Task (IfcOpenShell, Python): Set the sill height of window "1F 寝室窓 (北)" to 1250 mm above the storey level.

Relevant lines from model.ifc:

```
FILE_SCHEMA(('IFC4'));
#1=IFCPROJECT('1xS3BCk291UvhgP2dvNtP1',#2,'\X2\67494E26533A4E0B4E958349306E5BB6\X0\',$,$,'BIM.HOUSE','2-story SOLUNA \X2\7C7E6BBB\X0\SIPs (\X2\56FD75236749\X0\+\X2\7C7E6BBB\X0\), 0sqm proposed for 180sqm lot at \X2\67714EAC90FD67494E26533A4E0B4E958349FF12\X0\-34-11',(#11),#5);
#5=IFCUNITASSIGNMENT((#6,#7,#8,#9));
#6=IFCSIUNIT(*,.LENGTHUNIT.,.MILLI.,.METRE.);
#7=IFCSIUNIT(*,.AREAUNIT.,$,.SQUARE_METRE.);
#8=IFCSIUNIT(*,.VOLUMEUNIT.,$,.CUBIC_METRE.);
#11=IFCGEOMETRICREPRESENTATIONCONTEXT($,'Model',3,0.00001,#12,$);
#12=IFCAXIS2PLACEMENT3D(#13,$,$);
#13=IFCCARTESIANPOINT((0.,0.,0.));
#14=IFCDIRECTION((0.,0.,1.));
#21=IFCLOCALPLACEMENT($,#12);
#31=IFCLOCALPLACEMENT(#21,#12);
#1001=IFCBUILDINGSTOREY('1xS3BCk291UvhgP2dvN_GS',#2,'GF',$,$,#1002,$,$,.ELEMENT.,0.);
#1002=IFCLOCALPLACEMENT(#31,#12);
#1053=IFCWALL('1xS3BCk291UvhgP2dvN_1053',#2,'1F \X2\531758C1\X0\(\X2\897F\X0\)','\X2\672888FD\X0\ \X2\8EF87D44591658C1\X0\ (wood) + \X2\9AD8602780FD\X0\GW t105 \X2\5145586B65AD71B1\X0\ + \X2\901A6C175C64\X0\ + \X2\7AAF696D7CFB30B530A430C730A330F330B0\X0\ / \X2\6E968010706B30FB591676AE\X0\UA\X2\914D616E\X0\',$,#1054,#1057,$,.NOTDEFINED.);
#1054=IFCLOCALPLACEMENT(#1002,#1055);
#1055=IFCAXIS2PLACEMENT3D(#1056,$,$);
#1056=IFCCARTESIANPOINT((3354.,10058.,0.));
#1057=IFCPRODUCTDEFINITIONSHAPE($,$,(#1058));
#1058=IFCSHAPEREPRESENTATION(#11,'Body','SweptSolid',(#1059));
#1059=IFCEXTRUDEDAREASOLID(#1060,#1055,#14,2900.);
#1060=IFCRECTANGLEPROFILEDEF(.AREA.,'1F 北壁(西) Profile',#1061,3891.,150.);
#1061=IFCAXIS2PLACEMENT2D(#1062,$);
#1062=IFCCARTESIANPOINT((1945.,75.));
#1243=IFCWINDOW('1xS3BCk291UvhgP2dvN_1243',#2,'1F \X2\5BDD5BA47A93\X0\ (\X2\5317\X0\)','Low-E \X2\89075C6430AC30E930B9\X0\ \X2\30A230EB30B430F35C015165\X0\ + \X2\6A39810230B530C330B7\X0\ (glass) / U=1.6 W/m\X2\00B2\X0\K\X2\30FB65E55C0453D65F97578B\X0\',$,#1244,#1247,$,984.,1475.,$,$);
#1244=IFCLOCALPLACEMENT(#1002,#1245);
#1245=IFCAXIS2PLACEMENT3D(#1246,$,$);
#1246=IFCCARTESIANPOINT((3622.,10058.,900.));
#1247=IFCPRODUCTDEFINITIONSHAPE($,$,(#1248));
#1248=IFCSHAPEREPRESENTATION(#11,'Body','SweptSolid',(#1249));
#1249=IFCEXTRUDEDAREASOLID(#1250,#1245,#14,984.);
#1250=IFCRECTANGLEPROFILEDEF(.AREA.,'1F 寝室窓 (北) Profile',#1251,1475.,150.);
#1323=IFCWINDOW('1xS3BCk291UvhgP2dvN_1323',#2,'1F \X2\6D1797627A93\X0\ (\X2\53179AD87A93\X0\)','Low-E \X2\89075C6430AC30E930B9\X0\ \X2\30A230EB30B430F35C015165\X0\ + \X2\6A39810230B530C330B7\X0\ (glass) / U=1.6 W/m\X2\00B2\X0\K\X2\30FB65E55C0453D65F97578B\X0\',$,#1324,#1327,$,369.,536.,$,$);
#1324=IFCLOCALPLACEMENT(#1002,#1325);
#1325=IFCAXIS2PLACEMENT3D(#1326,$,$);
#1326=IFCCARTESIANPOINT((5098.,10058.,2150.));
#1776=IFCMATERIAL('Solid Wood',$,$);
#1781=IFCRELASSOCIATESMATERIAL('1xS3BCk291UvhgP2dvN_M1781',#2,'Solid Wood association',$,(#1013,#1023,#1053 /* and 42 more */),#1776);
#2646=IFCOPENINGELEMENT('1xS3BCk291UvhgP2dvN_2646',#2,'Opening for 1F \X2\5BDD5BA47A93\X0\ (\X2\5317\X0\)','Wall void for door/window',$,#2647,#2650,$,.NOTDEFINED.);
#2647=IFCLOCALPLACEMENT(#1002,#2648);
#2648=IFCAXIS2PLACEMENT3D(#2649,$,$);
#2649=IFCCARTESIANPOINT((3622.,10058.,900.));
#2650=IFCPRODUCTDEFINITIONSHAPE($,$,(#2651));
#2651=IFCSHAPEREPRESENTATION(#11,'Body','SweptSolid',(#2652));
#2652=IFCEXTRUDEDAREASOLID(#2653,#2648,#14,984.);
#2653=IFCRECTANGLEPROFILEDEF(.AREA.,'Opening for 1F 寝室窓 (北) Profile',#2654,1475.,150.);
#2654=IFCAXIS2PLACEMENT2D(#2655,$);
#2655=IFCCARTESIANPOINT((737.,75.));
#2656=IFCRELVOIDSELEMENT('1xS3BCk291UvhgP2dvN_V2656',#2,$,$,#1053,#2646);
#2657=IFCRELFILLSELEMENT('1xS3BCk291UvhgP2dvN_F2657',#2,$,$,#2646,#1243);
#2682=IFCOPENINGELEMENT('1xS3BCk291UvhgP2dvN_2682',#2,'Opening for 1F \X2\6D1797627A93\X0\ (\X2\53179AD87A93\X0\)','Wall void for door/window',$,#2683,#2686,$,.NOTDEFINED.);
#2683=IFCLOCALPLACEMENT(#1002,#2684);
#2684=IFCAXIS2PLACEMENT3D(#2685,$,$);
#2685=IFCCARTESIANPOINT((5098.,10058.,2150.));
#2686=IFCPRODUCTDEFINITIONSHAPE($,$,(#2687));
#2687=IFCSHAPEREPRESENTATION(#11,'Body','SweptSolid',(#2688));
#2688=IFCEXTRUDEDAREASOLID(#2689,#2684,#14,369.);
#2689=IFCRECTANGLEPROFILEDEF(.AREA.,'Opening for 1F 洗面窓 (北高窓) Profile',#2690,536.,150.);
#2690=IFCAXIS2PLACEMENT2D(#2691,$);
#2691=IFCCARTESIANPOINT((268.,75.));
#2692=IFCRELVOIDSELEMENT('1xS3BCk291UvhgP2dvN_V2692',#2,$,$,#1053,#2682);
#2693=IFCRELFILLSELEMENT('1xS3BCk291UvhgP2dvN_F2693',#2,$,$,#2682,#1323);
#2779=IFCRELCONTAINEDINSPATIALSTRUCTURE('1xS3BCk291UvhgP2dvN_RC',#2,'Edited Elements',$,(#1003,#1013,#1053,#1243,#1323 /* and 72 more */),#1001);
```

```python
import numpy as np
import ifcopenshell
import ifcopenshell.api.geometry
import ifcopenshell.geom
import ifcopenshell.util.element
import ifcopenshell.util.placement
import ifcopenshell.util.shape
import ifcopenshell.util.unit

model = ifcopenshell.open("model.ifc")
unit_scale = ifcopenshell.util.unit.calculate_unit_scale(model)

window = model.by_guid("1xS3BCk291UvhgP2dvN_1243")
opening = window.FillsVoids[0].RelatingOpeningElement
storey = ifcopenshell.util.element.get_container(window, ifc_class="IfcBuildingStorey")
level = ifcopenshell.util.placement.get_local_placement(storey.ObjectPlacement)[2, 3]

# The opening's origin need not be at the sill, so measure its lowest point.
shape = ifcopenshell.geom.create_shape(ifcopenshell.geom.settings(), opening)
bottom = ifcopenshell.util.shape.get_shape_bottom_elevation(shape, shape.geometry) / unit_scale
dz = level + 1250.0 - bottom

shift = np.array([0.0, 0.0, dz])
# The window is not placed relative to its opening, so move both.
for product in (opening, window):
    matrix = ifcopenshell.util.placement.get_local_placement(product.ObjectPlacement)
    matrix[:3, 3] += shift
    ifcopenshell.api.geometry.edit_object_placement(model, product=product, matrix=matrix, is_si=False)

print(f"moved by {dz * unit_scale:+.3f} m")

model.write("model-out.ifc")
```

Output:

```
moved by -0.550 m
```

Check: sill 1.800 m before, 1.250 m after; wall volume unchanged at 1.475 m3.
